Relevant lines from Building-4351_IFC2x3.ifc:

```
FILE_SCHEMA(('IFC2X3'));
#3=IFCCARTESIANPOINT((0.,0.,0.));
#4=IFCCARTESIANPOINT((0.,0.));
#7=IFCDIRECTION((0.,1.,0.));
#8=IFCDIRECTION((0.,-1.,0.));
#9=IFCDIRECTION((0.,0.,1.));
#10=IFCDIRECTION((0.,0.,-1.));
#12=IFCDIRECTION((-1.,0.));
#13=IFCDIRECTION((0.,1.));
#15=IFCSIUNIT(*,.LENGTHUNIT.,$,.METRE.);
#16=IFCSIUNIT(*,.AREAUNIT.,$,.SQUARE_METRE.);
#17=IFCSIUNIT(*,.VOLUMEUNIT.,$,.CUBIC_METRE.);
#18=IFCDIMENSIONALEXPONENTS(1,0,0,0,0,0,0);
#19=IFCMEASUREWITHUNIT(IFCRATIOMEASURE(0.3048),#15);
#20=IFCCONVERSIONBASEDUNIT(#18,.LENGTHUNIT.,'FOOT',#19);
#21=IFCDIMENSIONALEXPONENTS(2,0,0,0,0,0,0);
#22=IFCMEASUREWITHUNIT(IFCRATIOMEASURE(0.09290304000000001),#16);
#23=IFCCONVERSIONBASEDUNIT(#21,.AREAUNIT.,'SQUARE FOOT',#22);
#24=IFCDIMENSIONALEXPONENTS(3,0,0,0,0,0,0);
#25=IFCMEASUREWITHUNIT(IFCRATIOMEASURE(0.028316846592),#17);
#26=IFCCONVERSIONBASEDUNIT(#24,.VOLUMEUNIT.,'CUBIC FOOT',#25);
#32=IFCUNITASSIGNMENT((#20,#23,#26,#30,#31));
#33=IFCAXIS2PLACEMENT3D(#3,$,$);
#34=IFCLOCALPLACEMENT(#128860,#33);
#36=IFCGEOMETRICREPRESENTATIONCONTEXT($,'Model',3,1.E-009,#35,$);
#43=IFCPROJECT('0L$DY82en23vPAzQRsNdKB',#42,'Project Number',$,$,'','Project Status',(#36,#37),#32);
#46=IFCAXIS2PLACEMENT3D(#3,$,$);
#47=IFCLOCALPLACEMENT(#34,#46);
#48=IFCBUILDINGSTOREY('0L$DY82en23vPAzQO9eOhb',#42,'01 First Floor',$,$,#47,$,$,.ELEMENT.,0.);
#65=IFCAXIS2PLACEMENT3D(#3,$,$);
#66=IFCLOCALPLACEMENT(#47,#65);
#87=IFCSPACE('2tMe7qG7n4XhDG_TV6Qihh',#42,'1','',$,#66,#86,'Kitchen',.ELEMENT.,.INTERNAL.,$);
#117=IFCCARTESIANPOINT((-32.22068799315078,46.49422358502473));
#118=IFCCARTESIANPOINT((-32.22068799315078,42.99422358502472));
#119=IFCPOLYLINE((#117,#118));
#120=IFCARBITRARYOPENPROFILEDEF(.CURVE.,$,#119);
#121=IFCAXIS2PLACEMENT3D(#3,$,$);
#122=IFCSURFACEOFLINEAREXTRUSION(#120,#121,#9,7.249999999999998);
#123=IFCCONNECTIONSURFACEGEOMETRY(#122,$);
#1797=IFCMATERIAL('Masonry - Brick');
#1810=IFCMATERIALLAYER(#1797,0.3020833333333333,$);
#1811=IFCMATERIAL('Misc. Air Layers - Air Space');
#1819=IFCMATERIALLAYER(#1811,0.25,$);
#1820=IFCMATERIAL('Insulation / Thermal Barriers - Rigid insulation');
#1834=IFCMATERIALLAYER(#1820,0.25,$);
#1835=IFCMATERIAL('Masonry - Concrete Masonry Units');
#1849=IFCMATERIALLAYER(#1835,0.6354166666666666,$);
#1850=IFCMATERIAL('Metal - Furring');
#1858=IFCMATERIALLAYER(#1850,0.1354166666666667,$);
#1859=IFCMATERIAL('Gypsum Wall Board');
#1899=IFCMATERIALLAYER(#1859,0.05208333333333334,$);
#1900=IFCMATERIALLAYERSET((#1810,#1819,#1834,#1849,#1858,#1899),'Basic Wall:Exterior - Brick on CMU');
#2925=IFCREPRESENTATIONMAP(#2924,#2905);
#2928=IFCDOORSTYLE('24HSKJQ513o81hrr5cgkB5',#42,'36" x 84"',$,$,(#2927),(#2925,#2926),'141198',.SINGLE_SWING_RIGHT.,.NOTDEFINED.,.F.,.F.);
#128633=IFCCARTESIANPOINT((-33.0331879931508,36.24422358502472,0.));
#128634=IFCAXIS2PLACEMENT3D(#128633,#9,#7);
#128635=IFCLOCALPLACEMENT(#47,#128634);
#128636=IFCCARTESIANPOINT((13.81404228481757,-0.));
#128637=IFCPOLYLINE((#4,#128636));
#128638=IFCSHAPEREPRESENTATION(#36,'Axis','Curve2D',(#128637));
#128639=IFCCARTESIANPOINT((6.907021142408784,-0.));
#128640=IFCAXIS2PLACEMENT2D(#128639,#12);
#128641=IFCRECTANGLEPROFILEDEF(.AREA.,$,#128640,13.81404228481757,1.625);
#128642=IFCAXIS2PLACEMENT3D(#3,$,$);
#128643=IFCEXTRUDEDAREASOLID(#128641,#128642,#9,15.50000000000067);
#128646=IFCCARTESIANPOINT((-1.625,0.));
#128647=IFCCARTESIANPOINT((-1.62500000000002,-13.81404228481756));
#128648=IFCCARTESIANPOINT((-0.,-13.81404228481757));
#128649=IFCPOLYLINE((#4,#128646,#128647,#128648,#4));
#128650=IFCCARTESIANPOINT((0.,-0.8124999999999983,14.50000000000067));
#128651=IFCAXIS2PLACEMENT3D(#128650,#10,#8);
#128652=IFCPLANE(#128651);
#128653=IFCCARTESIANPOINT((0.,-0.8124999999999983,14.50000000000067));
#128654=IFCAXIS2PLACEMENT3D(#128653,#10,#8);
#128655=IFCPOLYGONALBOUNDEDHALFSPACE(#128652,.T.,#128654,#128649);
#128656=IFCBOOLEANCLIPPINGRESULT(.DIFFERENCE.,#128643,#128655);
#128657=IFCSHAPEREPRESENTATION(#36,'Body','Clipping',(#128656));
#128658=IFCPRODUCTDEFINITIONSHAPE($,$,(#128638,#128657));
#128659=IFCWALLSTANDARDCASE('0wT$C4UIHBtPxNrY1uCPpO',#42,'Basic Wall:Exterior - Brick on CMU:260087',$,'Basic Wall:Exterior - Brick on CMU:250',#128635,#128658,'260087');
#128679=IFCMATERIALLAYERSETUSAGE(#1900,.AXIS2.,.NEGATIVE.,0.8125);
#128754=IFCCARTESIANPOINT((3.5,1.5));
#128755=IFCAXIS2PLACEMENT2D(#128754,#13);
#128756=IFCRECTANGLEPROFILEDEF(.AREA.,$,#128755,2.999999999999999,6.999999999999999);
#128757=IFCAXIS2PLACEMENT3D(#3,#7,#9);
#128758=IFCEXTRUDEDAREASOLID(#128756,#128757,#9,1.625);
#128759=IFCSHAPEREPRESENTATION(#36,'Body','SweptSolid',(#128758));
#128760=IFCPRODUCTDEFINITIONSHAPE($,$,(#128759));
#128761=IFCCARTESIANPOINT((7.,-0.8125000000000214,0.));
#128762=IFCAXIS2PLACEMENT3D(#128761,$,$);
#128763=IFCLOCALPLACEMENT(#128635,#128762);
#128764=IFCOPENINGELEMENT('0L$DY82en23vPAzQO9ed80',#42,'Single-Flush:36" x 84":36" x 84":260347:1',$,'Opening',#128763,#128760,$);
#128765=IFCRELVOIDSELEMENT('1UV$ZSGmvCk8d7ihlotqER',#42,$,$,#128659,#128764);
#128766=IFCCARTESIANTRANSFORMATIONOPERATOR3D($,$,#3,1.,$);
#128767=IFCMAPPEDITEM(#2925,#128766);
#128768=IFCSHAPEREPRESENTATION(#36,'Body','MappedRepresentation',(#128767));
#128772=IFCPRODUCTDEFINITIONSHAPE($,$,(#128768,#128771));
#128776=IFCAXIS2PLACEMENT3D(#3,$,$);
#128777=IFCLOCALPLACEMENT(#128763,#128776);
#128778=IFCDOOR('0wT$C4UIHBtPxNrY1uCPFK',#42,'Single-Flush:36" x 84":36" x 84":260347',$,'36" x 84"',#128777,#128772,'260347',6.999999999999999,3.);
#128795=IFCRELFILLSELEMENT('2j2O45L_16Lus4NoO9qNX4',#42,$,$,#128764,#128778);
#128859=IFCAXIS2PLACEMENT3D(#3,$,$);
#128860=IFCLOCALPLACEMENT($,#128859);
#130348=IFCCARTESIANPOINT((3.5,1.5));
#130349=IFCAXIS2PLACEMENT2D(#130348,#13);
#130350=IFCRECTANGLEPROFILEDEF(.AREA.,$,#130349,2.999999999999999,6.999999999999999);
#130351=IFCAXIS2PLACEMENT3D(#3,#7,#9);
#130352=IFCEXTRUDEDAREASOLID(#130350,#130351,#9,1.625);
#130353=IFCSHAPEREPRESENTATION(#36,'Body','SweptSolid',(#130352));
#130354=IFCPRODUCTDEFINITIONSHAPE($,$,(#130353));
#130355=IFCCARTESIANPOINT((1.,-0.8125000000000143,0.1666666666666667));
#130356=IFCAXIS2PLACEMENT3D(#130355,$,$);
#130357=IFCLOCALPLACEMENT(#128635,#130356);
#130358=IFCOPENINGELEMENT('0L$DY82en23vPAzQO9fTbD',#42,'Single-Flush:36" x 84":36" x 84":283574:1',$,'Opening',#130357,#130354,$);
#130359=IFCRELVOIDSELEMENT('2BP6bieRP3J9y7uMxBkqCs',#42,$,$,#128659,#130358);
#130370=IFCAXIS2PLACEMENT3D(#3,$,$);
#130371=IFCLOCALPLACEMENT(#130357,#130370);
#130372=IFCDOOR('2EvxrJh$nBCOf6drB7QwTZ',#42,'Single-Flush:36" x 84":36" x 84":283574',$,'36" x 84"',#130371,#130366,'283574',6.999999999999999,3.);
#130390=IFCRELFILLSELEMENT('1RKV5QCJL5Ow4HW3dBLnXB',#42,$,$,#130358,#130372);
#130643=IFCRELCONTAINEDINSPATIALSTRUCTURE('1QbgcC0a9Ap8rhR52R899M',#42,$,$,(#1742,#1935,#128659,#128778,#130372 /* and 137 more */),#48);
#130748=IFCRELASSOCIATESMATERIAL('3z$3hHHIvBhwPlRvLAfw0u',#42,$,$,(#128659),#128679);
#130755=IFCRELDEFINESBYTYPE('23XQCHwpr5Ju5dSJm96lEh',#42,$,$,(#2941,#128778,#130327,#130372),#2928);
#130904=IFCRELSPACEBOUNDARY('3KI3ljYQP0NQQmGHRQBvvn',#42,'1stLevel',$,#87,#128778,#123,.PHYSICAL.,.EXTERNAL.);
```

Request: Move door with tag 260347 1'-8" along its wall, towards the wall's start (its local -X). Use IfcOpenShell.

```python
import numpy as np
import ifcopenshell
import ifcopenshell.api.geometry
import ifcopenshell.util.placement
import ifcopenshell.util.unit

model = ifcopenshell.open("Building-4351_IFC2x3.ifc")
unit_scale = ifcopenshell.util.unit.calculate_unit_scale(model)

door = model.by_guid("0wT$C4UIHBtPxNrY1uCPFK")
opening = door.FillsVoids[0].RelatingOpeningElement
wall = opening.VoidsElements[0].RelatingBuildingElement

wall_matrix = ifcopenshell.util.placement.get_local_placement(wall.ObjectPlacement)
shift = wall_matrix[:3, 0] * -20 * 0.0254 / unit_scale
before = ifcopenshell.util.placement.get_local_placement(door.ObjectPlacement)[:3, 3].copy()

# The door is placed relative to its opening, so it follows when the opening moves.
matrix = ifcopenshell.util.placement.get_local_placement(opening.ObjectPlacement)
matrix[:3, 3] += shift
ifcopenshell.api.geometry.edit_object_placement(
    model, product=opening, matrix=matrix, is_si=False, should_transform_children=True
)

# Space boundary surfaces are stored in each space's coordinates; move them too.
for rel in door.ProvidesBoundaries:
    if not rel.ConnectionGeometry:
        continue
    surface = rel.ConnectionGeometry.SurfaceOnRelatingElement
    space_matrix = ifcopenshell.util.placement.get_local_placement(rel.RelatingSpace.ObjectPlacement)
    point = np.array(surface.Position.Location.Coordinates) + space_matrix[:3, :3].T @ shift
    surface.Position = model.createIfcAxis2Placement3D(
        model.createIfcCartesianPoint(point.tolist()), surface.Position.Axis, surface.Position.RefDirection
    )

after = ifcopenshell.util.placement.get_local_placement(door.ObjectPlacement)[:3, 3]
print("door moved by", (after - before).round(3) + 0.0)

model.write("Building-4351_IFC2x3_updated.ifc")
```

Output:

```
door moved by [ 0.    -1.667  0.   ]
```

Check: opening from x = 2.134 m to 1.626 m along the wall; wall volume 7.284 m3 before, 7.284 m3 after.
